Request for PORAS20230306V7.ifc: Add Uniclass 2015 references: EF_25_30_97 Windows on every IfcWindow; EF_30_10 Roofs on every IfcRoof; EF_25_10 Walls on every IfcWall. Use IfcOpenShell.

First a look at what the model holds.

```python
import ifcopenshell

model = ifcopenshell.open("PORAS20230306V7.ifc")
print(model.schema)
print("classifications:", [c.Name for c in model.by_type("IfcClassification")])
for ifc_class in ("IfcDoor", "IfcRoof", "IfcStair", "IfcWall", "IfcWindow"):
    print(ifc_class, len(model.by_type(ifc_class)))
```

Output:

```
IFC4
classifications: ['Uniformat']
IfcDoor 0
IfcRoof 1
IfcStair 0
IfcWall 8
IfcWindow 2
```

```python
import ifcopenshell
import ifcopenshell.api.classification

model = ifcopenshell.open("PORAS20230306V7.ifc")

system = ifcopenshell.api.classification.add_classification(model, classification="Uniclass 2015")

codes = {
    "IfcWindow": ("EF_25_30_97", "Windows"),
    "IfcRoof": ("EF_30_10", "Roofs"),
    "IfcWall": ("EF_25_10", "Walls"),
}
for ifc_class, (code, name) in codes.items():
    products = model.by_type(ifc_class)
    ifcopenshell.api.classification.add_reference(
        model, products=products, classification=system, identification=code, name=name
    )
    print(code, len(products))

model.write("PORAS20230306V7_updated.ifc")
```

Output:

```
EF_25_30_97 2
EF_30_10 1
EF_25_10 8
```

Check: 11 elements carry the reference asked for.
